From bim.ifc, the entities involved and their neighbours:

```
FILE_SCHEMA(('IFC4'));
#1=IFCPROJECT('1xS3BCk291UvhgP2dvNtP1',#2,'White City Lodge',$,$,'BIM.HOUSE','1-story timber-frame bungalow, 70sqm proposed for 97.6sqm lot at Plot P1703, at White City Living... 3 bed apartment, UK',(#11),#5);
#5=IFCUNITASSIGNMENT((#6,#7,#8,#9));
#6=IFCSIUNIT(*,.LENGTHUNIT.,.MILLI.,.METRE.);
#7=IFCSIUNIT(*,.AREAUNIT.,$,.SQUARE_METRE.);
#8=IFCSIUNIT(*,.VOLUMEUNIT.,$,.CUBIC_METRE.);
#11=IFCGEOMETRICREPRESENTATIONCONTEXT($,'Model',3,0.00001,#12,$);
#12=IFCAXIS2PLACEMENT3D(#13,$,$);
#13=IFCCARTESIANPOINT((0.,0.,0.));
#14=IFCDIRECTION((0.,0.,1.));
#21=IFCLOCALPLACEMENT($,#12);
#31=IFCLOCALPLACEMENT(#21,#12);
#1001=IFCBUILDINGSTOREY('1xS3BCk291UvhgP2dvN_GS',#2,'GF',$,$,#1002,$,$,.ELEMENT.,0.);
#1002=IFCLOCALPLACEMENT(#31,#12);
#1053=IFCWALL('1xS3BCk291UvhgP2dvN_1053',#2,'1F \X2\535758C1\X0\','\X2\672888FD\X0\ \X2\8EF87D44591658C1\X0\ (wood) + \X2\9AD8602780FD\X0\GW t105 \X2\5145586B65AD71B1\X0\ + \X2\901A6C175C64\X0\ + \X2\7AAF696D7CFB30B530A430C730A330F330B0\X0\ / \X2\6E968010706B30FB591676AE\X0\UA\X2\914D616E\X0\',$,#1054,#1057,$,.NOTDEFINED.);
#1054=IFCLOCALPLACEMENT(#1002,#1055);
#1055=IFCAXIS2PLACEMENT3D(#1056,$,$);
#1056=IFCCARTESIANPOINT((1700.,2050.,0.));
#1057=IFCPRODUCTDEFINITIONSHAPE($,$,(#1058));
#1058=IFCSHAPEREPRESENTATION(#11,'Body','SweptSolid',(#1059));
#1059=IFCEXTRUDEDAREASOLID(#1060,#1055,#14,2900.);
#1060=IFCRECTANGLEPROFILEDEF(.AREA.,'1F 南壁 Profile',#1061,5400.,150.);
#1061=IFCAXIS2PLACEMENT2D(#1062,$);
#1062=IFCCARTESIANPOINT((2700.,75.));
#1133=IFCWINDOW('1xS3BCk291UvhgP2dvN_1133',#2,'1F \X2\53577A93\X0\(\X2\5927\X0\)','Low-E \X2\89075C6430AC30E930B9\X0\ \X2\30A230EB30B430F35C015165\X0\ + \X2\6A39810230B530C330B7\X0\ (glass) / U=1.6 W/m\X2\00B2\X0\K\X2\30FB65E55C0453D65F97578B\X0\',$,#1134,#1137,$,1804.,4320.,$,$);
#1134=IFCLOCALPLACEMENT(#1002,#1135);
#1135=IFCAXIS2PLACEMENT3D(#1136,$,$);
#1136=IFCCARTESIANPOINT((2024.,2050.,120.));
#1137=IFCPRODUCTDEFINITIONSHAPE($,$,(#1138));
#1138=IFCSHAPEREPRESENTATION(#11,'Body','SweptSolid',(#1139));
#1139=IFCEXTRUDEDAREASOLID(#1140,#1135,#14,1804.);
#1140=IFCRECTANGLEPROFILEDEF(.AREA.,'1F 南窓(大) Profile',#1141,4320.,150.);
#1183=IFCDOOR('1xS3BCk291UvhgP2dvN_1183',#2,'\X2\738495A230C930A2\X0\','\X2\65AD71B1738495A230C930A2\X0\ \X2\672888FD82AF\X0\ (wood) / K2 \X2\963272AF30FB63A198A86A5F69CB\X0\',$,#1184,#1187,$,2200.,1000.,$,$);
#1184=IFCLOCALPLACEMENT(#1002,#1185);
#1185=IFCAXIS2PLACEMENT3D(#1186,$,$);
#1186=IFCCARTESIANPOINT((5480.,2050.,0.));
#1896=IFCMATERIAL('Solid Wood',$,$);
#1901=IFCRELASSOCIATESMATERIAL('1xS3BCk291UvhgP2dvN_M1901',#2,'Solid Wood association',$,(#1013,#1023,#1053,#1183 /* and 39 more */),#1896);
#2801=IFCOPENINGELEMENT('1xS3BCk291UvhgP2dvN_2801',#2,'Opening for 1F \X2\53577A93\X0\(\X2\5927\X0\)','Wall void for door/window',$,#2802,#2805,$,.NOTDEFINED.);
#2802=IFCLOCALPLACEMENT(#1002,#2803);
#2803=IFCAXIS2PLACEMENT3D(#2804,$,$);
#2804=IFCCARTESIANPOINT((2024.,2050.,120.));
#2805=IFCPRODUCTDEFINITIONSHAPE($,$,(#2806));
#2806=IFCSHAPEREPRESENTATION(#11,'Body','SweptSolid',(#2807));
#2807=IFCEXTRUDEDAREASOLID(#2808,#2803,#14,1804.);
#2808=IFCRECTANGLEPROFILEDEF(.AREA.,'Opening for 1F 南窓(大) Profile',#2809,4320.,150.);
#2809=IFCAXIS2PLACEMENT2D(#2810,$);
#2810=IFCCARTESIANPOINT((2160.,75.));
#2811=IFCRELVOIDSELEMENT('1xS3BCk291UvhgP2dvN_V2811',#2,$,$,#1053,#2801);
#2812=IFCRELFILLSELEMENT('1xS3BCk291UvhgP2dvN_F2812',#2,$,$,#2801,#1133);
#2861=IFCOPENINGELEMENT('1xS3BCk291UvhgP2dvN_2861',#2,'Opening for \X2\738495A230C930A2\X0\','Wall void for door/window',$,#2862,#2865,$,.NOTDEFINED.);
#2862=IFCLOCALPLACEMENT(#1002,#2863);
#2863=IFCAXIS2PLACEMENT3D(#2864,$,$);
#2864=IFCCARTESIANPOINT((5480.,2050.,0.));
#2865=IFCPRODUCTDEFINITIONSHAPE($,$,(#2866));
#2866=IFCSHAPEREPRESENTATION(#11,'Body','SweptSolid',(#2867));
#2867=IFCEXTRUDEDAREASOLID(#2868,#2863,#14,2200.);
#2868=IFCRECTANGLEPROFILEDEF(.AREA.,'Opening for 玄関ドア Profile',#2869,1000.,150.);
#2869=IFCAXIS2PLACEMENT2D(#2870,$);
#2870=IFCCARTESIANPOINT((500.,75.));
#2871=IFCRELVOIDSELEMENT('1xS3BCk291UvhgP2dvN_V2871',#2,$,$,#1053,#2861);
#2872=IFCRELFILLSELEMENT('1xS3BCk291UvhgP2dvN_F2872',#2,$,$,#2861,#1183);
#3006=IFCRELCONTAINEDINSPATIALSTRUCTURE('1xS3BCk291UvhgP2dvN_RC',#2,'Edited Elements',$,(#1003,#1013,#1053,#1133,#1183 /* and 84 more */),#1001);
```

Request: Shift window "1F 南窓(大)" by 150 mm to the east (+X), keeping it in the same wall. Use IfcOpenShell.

```python
import ifcopenshell
import ifcopenshell.api.geometry
import ifcopenshell.util.placement

model = ifcopenshell.open("bim.ifc")

window = model.by_id(1133)
opening = window.FillsVoids[0].RelatingOpeningElement
wall = opening.VoidsElements[0].RelatingBuildingElement

wall_matrix = ifcopenshell.util.placement.get_local_placement(wall.ObjectPlacement)
shift = wall_matrix[:3, 0] * 150.0
before = ifcopenshell.util.placement.get_local_placement(window.ObjectPlacement)[:3, 3].copy()

# The window is not placed relative to its opening, so move both.
for product in (opening, window):
    matrix = ifcopenshell.util.placement.get_local_placement(product.ObjectPlacement)
    matrix[:3, 3] += shift
    ifcopenshell.api.geometry.edit_object_placement(model, product=product, matrix=matrix, is_si=False)

after = ifcopenshell.util.placement.get_local_placement(window.ObjectPlacement)[:3, 3]
print("window moved by", (after - before).round(3) + 0.0)

model.write("bim_updated.ifc")
```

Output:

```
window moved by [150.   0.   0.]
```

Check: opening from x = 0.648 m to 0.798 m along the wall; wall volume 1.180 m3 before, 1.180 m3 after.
